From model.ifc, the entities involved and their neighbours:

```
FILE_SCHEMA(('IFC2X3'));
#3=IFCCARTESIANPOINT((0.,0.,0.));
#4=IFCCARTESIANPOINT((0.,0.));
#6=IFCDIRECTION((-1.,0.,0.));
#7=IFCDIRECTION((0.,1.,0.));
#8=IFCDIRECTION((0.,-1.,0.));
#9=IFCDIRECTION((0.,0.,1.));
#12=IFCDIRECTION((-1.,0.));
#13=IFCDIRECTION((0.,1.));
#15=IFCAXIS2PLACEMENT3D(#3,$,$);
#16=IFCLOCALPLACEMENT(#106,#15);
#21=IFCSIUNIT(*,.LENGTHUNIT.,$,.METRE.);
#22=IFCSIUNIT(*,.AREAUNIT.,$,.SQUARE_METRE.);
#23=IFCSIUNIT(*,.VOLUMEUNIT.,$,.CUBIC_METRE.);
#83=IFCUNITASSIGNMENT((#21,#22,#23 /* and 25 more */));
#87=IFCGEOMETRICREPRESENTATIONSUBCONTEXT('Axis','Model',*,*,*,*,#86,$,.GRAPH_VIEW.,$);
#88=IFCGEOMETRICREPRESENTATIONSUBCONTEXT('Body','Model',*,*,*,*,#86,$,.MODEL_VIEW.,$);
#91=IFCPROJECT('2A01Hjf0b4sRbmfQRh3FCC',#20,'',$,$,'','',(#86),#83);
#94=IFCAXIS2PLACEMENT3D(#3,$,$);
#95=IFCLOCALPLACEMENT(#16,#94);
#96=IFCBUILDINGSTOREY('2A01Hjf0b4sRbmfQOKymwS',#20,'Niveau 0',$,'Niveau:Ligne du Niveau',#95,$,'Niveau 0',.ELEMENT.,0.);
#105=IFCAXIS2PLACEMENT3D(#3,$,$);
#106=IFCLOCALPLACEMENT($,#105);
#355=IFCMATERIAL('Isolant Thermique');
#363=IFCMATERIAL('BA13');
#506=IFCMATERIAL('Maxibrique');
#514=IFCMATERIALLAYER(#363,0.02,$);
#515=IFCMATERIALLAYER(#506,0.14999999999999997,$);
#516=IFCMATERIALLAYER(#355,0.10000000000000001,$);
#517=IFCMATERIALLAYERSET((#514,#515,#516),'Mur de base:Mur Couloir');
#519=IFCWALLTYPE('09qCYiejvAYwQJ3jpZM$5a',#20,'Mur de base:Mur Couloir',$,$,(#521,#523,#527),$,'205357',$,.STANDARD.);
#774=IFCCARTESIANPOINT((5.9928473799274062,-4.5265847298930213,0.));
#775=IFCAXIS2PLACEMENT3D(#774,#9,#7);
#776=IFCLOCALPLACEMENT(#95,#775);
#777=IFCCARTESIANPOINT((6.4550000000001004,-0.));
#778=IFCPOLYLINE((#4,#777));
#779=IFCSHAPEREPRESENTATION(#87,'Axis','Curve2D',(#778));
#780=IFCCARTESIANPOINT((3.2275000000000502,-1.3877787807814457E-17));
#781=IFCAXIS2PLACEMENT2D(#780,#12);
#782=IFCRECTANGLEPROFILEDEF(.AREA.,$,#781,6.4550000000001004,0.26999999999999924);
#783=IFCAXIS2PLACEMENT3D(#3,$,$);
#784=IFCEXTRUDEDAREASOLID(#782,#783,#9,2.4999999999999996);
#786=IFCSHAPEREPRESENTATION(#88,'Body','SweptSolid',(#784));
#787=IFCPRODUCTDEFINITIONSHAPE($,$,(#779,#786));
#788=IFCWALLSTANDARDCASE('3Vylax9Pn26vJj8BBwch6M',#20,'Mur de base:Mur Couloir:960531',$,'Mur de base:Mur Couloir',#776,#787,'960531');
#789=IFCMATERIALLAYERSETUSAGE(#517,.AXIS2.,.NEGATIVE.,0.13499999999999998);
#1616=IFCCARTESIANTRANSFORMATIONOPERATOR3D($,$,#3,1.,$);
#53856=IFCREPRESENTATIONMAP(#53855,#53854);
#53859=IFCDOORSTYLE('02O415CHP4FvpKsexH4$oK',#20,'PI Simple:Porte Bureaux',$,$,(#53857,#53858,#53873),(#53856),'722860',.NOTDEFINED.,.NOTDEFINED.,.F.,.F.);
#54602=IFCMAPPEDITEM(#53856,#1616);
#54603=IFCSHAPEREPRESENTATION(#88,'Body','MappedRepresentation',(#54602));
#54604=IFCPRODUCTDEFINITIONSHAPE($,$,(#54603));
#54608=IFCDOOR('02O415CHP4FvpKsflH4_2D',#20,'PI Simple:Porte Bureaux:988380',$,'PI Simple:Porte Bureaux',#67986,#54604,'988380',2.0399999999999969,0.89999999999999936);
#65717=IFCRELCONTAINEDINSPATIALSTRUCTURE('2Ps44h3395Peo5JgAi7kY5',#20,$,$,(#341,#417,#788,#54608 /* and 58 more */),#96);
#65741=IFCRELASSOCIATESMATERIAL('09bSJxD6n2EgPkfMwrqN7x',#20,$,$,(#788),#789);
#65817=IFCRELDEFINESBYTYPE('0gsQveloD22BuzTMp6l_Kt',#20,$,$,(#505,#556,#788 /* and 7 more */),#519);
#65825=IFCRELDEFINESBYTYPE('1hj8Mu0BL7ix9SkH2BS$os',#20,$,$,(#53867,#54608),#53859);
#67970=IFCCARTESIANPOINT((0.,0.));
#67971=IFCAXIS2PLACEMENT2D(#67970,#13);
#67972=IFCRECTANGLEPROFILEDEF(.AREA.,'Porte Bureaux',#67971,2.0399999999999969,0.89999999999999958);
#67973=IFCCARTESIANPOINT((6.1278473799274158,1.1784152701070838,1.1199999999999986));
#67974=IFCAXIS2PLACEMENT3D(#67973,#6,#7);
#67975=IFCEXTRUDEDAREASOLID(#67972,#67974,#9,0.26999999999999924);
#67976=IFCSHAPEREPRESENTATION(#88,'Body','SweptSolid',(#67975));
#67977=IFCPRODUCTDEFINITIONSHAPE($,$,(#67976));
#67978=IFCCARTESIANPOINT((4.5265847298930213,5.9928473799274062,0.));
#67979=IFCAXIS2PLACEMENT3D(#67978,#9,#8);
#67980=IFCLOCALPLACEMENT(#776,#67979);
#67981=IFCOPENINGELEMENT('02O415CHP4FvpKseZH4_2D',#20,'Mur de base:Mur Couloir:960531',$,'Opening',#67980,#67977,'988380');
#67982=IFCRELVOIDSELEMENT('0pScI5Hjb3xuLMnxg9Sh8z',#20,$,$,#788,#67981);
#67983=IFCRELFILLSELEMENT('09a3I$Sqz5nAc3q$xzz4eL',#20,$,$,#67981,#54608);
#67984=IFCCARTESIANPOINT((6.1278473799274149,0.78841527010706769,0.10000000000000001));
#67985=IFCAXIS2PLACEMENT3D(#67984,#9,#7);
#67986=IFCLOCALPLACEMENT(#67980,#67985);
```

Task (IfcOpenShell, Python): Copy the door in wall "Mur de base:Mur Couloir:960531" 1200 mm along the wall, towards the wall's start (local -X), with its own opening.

```python
import ifcopenshell
import ifcopenshell.api.feature
import ifcopenshell.api.geometry
import ifcopenshell.api.root
import ifcopenshell.geom
import ifcopenshell.util.element
import ifcopenshell.util.placement
import ifcopenshell.util.shape

model = ifcopenshell.open("model.ifc")
settings = ifcopenshell.geom.settings()


def volume(element):
    """Net volume in cubic metres, openings subtracted."""
    shape = ifcopenshell.geom.create_shape(settings, element)
    return ifcopenshell.util.shape.get_volume(shape.geometry)


def reuse_history(source, copy):
    """copy_class also copies each property set's owner history, people and application; keep the originals."""
    for rel in copy.IsDefinedBy:
        if rel.is_a("IfcRelDefinesByProperties") and (history := rel.RelatingPropertyDefinition.OwnerHistory):
            rel.RelatingPropertyDefinition.OwnerHistory = source.OwnerHistory
            ifcopenshell.util.element.remove_deep2(model, history)


door = model.by_guid("02O415CHP4FvpKsflH4_2D")
opening = door.FillsVoids[0].RelatingOpeningElement
wall = opening.VoidsElements[0].RelatingBuildingElement
before = volume(wall)
shift = ifcopenshell.util.placement.get_local_placement(wall.ObjectPlacement)[:3, 0] * -1.2

# copy_class copies the void relationship, type, container and properties, but no geometry.
new_opening = ifcopenshell.api.root.copy_class(model, product=opening)
new_opening.Representation = ifcopenshell.util.element.copy_deep(
    model, opening.Representation, exclude=["IfcGeometricRepresentationContext", "IfcRepresentationMap"]
)
new_opening.Name = "Mur de base:Mur Couloir"
new_opening.Tag = None
new_door = ifcopenshell.api.root.copy_class(model, product=door)
new_door.Representation = ifcopenshell.util.element.copy_deep(
    model, door.Representation, exclude=["IfcGeometricRepresentationContext", "IfcRepresentationMap"]
)
new_door.Name = "PI Simple:Porte Bureaux"
new_door.Tag = None
reuse_history(door, new_door)
fills = ifcopenshell.api.feature.add_filling(model, opening=new_opening, element=new_door)
fills.OwnerHistory = new_door.OwnerHistory  # required in IFC2X3

for old, new in ((opening, new_opening), (door, new_door)):
    matrix = ifcopenshell.util.placement.get_local_placement(old.ObjectPlacement)
    matrix[:3, 3] += shift
    ifcopenshell.api.geometry.edit_object_placement(model, product=new, matrix=matrix, is_si=False)

after = volume(wall)

print(f"wall volume {before:.3f} -> {after:.3f} m3")

model.write("model_v2.ifc")
```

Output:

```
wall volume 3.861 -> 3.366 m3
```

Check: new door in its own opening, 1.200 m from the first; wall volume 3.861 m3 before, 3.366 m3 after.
